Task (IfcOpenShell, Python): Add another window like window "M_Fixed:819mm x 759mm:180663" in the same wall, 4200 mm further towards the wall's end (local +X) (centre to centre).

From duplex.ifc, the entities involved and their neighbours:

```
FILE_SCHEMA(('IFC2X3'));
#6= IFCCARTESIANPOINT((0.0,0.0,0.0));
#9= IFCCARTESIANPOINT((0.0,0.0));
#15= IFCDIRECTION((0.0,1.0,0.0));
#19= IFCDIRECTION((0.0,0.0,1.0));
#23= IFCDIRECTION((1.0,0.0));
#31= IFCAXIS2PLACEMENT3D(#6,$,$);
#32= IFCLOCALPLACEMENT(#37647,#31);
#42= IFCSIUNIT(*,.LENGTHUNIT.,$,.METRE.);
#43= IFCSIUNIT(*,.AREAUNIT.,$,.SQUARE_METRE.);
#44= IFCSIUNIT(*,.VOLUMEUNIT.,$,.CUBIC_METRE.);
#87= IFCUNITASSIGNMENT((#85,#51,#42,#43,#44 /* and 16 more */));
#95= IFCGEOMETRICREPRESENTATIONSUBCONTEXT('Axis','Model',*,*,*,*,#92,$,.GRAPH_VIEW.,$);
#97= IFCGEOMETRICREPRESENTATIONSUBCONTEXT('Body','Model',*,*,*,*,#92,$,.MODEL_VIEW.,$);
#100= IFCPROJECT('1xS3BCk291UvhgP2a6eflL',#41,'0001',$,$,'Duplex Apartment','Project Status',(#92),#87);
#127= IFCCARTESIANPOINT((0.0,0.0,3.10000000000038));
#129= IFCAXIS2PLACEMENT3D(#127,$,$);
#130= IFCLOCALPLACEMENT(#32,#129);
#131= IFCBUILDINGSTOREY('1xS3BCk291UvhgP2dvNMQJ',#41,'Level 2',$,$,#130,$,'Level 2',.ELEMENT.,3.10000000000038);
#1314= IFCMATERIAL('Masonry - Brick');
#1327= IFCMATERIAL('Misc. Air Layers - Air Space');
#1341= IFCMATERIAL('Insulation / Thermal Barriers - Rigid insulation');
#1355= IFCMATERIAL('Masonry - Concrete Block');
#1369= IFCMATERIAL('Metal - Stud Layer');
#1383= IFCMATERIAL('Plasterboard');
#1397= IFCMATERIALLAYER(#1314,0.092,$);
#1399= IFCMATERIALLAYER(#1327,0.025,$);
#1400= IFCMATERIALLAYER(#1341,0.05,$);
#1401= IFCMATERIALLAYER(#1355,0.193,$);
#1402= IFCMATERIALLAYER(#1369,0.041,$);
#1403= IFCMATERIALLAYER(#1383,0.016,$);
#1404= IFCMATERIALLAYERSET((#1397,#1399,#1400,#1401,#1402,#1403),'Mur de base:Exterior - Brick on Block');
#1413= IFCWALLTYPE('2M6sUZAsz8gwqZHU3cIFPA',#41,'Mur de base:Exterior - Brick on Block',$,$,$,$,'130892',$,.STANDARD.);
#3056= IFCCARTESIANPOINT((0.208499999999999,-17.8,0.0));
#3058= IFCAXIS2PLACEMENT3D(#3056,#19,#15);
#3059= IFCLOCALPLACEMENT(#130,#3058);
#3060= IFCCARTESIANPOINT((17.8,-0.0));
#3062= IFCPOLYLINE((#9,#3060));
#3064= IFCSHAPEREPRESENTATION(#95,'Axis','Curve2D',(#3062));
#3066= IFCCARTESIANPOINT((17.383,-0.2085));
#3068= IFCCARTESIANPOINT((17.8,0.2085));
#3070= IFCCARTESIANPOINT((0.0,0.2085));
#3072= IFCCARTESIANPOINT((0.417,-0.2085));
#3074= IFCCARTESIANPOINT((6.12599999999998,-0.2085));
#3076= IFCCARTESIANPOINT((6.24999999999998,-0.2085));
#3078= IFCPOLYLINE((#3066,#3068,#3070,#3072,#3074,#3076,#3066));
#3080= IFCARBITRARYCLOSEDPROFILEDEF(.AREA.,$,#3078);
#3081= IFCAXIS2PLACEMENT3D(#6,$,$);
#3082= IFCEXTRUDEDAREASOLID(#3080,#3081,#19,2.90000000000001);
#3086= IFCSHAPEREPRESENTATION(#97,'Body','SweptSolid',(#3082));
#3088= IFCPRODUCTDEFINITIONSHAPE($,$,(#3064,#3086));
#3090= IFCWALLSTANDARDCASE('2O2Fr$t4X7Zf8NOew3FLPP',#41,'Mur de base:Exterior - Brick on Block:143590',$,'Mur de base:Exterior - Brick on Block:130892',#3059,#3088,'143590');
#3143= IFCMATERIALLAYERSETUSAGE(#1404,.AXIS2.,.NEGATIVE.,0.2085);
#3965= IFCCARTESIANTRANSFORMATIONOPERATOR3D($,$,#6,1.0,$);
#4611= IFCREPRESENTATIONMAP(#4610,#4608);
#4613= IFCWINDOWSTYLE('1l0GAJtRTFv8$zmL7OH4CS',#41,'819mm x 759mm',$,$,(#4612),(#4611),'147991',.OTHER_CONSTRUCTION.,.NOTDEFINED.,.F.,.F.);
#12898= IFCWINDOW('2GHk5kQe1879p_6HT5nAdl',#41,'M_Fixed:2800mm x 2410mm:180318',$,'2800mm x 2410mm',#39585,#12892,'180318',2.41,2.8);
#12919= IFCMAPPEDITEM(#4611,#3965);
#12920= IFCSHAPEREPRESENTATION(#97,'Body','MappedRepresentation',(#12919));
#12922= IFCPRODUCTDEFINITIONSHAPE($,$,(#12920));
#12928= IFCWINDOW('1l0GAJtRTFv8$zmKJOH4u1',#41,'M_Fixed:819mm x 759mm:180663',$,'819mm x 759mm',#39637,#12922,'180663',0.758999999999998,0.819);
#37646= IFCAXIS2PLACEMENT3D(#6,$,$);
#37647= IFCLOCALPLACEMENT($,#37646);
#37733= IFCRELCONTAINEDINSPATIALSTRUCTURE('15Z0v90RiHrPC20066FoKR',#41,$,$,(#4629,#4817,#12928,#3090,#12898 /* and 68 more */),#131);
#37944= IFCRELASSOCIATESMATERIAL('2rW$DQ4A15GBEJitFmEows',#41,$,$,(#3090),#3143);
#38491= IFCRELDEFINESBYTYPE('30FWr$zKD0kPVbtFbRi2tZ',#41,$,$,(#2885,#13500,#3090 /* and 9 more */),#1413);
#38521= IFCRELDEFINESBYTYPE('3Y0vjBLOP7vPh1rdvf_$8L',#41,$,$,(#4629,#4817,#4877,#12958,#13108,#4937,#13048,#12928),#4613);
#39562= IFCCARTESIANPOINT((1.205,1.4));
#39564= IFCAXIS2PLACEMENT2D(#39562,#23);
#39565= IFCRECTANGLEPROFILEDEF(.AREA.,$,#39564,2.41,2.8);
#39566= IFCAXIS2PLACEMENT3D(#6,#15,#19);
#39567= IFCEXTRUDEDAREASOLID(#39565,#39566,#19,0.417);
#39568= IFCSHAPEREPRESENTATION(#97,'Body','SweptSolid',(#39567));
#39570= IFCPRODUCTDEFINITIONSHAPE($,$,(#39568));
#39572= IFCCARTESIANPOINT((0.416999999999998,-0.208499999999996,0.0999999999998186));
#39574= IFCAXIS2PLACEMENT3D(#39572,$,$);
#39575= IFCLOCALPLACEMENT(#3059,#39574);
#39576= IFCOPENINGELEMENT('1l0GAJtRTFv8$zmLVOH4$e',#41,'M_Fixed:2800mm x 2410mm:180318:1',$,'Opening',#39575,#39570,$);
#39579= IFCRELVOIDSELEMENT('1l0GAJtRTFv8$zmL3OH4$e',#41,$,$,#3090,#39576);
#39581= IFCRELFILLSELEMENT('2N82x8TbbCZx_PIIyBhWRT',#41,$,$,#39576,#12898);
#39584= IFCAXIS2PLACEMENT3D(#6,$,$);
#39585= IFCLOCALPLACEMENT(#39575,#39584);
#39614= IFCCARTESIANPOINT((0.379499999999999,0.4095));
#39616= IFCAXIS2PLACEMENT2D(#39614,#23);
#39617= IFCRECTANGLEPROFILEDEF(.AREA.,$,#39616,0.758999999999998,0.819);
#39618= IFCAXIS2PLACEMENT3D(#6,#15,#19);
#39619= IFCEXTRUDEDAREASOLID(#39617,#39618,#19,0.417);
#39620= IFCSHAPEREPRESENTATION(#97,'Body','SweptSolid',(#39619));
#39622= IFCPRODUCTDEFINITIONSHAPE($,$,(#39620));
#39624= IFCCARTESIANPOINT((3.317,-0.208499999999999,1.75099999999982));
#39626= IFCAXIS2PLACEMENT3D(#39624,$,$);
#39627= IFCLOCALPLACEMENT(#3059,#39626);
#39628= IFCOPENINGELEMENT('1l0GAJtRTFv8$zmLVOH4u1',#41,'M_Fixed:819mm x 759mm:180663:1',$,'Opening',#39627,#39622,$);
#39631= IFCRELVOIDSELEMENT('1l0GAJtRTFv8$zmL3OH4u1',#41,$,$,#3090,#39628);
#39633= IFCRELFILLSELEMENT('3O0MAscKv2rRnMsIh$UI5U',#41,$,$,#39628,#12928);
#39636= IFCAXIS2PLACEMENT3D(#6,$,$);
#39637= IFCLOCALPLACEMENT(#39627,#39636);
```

```python
import ifcopenshell
import ifcopenshell.api.feature
import ifcopenshell.api.geometry
import ifcopenshell.api.root
import ifcopenshell.geom
import ifcopenshell.util.element
import ifcopenshell.util.placement
import ifcopenshell.util.shape

model = ifcopenshell.open("duplex.ifc")
settings = ifcopenshell.geom.settings()


def volume(element):
    """Net volume in cubic metres, openings subtracted."""
    shape = ifcopenshell.geom.create_shape(settings, element)
    return ifcopenshell.util.shape.get_volume(shape.geometry)


def reuse_history(source, copy):
    """copy_class also copies each property set's owner history, people and application; keep the originals."""
    for rel in copy.IsDefinedBy:
        if rel.is_a("IfcRelDefinesByProperties") and (history := rel.RelatingPropertyDefinition.OwnerHistory):
            rel.RelatingPropertyDefinition.OwnerHistory = source.OwnerHistory
            ifcopenshell.util.element.remove_deep2(model, history)


window = model.by_id(12928)
opening = window.FillsVoids[0].RelatingOpeningElement
wall = opening.VoidsElements[0].RelatingBuildingElement
before = volume(wall)
shift = ifcopenshell.util.placement.get_local_placement(wall.ObjectPlacement)[:3, 0] * 4.2

# copy_class copies the void relationship, type, container and properties, but no geometry.
new_opening = ifcopenshell.api.root.copy_class(model, product=opening)
new_opening.Representation = ifcopenshell.util.element.copy_deep(
    model, opening.Representation, exclude=["IfcGeometricRepresentationContext", "IfcRepresentationMap"]
)
new_opening.Name = "M_Fixed:819mm x 759mm"
new_window = ifcopenshell.api.root.copy_class(model, product=window)
new_window.Representation = ifcopenshell.util.element.copy_deep(
    model, window.Representation, exclude=["IfcGeometricRepresentationContext", "IfcRepresentationMap"]
)
new_window.Name = "M_Fixed:819mm x 759mm"
new_window.Tag = None
reuse_history(window, new_window)
fills = ifcopenshell.api.feature.add_filling(model, opening=new_opening, element=new_window)
fills.OwnerHistory = new_window.OwnerHistory  # required in IFC2X3

for old, new in ((opening, new_opening), (window, new_window)):
    matrix = ifcopenshell.util.placement.get_local_placement(old.ObjectPlacement)
    matrix[:3, 3] += shift
    ifcopenshell.api.geometry.edit_object_placement(model, product=new, matrix=matrix, is_si=False)

after = volume(wall)

print(f"wall volume {before:.3f} -> {after:.3f} m3")

model.write("duplex_v2.ifc")
```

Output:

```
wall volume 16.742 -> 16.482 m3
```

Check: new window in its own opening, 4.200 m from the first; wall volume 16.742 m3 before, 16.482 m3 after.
